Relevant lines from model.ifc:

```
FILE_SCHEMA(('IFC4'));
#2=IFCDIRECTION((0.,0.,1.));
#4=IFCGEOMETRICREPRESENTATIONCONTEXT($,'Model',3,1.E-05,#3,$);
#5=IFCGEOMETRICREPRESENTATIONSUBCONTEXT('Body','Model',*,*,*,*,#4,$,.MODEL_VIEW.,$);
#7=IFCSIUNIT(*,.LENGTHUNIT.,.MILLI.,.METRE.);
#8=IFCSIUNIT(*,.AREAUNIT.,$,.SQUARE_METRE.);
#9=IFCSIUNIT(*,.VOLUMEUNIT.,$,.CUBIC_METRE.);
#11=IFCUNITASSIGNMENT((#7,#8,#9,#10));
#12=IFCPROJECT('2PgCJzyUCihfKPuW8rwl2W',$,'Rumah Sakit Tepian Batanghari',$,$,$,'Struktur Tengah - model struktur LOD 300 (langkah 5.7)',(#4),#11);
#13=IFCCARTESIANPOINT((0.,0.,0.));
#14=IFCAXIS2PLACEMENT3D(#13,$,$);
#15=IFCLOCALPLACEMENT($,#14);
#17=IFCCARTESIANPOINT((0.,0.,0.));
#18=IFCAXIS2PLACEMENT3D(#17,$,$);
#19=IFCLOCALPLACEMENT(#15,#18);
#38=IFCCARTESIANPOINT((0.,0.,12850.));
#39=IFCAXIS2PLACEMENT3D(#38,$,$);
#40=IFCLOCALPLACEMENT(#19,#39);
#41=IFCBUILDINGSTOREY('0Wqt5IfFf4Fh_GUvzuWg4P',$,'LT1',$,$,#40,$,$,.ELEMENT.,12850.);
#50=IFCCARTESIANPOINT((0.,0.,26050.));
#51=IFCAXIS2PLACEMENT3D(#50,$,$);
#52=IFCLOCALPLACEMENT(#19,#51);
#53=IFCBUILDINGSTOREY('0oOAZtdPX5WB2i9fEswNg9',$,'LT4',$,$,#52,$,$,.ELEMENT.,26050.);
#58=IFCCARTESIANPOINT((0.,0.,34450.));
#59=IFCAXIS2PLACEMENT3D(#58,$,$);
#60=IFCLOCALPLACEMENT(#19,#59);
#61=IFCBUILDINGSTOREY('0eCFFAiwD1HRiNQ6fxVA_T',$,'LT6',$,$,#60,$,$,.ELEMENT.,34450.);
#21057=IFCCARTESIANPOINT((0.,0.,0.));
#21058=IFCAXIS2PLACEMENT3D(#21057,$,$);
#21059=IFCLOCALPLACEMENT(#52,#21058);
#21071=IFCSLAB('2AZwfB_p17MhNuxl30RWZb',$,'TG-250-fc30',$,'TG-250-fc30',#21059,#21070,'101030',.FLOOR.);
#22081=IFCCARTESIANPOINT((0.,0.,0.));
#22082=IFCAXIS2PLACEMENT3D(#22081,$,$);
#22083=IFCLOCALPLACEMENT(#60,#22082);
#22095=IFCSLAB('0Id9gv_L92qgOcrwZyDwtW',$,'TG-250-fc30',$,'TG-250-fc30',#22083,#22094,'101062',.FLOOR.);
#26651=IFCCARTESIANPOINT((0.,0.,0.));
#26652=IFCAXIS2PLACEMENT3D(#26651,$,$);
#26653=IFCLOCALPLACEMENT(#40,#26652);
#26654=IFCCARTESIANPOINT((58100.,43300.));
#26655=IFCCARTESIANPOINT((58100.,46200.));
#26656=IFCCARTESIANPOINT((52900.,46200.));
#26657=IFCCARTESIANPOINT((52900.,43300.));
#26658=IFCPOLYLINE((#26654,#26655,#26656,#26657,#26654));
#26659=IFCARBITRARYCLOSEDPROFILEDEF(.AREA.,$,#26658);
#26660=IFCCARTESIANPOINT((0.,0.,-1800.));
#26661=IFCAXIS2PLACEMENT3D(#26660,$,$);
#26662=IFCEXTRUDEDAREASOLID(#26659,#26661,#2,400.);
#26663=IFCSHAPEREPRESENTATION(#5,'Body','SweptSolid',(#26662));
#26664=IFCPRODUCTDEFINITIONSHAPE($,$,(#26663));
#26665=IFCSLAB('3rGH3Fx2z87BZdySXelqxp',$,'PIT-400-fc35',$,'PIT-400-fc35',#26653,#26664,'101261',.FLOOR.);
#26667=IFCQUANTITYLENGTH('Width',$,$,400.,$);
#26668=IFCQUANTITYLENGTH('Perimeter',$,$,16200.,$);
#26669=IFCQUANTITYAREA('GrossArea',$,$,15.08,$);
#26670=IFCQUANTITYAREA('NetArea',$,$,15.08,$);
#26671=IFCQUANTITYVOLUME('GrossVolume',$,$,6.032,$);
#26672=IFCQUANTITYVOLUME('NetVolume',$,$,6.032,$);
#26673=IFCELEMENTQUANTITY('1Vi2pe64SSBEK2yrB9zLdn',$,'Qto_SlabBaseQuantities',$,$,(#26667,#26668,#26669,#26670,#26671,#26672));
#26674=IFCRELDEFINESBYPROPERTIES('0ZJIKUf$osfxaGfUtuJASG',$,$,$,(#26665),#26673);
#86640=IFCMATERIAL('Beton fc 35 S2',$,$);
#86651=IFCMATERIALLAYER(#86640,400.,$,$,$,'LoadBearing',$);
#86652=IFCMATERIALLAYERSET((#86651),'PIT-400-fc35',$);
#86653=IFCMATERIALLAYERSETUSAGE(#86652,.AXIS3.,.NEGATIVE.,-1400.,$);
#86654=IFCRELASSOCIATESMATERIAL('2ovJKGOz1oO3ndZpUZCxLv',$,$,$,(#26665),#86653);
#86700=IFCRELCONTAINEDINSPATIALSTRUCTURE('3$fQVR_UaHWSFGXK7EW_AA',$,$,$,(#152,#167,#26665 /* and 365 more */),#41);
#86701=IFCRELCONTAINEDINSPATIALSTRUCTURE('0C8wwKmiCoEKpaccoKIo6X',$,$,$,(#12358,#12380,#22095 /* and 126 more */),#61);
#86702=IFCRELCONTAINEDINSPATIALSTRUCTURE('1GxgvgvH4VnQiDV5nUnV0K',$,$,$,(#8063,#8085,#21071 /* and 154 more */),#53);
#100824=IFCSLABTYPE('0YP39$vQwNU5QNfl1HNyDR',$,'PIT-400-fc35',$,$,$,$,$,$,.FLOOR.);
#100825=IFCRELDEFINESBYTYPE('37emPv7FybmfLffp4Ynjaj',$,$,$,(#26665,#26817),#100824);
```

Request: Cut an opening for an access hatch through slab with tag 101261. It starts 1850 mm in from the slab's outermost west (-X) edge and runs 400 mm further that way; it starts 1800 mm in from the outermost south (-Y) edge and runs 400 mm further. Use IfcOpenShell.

```python
import numpy as np
import ifcopenshell
import ifcopenshell.api.feature
import ifcopenshell.api.geometry
import ifcopenshell.api.pset
import ifcopenshell.api.root
import ifcopenshell.geom
import ifcopenshell.util.element
import ifcopenshell.util.placement
import ifcopenshell.util.representation
import ifcopenshell.util.shape
import ifcopenshell.util.unit

model = ifcopenshell.open("model.ifc")
unit_scale = ifcopenshell.util.unit.calculate_unit_scale(model)
area_scale = ifcopenshell.util.unit.calculate_unit_scale(model, "AREAUNIT")
volume_scale = ifcopenshell.util.unit.calculate_unit_scale(model, "VOLUMEUNIT")
settings = ifcopenshell.geom.settings()


def volume(element):
    """Net volume in cubic metres, openings subtracted."""
    shape = ifcopenshell.geom.create_shape(settings, element)
    return ifcopenshell.util.shape.get_volume(shape.geometry)


slab = model.by_guid("3rGH3Fx2z87BZdySXelqxp")
before = volume(slab)

# Extent in the slab's own axes, in metres. The edges named are its -X and -Y sides.
slab_shape = ifcopenshell.geom.create_shape(settings, slab)
vertices = ifcopenshell.util.shape.get_vertices(slab_shape.geometry)
x_min, y_min, bottom = vertices.min(axis=0)
top = vertices[:, 2].max()

opening = ifcopenshell.api.root.create_entity(model, ifc_class="IfcOpeningElement", name="Access hatch opening", predefined_type="OPENING")
context = ifcopenshell.util.representation.get_context(model, "Model", "Body", "MODEL_VIEW")
width, depth = 0.4, 0.4
outline = [(0.0, 0.0), (width, 0.0), (width, depth), (0.0, depth), (0.0, 0.0)]
# Overshoot both faces by 50 mm so the cut is clean.
shape = ifcopenshell.api.geometry.add_slab_representation(
    model, context=context, depth=top - bottom + 0.1, polyline=outline
)
ifcopenshell.api.geometry.assign_representation(model, product=opening, representation=shape)

matrix = ifcopenshell.util.placement.get_local_placement(slab.ObjectPlacement)
matrix[:, 3] = matrix @ np.append(np.array([x_min + 1.85, y_min + 1.8, bottom - 0.05]) / unit_scale, 1.0)
ifcopenshell.api.geometry.edit_object_placement(model, product=opening, matrix=matrix, is_si=False)
ifcopenshell.api.feature.add_feature(model, feature=opening, element=slab)

after = volume(slab)

# Update the slab's stored quantities.
qto = model.by_id(ifcopenshell.util.element.get_pset(slab, "Qto_SlabBaseQuantities", should_inherit=False)["id"])
ifcopenshell.api.pset.edit_qto(model, qto=qto, properties={
    "NetArea": after / (top - bottom) / area_scale,
    "NetVolume": after / volume_scale,
})

print(f"slab volume {before:.3f} -> {after:.3f} m3")

model.write("model_v2.ifc")
```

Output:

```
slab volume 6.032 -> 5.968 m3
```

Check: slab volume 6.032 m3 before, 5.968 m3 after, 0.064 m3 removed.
